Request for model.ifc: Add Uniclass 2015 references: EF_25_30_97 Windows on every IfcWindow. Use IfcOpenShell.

First a look at what the model holds.

```python
import ifcopenshell

model = ifcopenshell.open("model.ifc")
print(model.schema)
print("classifications:", [c.Name for c in model.by_type("IfcClassification")])
for ifc_class in ("IfcDoor", "IfcRoof", "IfcStair", "IfcWall", "IfcWindow"):
    print(ifc_class, len(model.by_type(ifc_class)))
```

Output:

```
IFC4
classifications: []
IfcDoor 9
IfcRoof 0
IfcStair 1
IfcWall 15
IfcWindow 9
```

```python
import ifcopenshell
import ifcopenshell.api.classification

model = ifcopenshell.open("model.ifc")

system = ifcopenshell.api.classification.add_classification(model, classification="Uniclass 2015")

codes = {
    "IfcWindow": ("EF_25_30_97", "Windows"),
}
for ifc_class, (code, name) in codes.items():
    products = model.by_type(ifc_class)
    ifcopenshell.api.classification.add_reference(
        model, products=products, classification=system, identification=code, name=name
    )
    print(code, len(products))

model.write("model_edited.ifc")
```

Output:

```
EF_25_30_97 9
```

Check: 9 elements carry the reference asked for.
